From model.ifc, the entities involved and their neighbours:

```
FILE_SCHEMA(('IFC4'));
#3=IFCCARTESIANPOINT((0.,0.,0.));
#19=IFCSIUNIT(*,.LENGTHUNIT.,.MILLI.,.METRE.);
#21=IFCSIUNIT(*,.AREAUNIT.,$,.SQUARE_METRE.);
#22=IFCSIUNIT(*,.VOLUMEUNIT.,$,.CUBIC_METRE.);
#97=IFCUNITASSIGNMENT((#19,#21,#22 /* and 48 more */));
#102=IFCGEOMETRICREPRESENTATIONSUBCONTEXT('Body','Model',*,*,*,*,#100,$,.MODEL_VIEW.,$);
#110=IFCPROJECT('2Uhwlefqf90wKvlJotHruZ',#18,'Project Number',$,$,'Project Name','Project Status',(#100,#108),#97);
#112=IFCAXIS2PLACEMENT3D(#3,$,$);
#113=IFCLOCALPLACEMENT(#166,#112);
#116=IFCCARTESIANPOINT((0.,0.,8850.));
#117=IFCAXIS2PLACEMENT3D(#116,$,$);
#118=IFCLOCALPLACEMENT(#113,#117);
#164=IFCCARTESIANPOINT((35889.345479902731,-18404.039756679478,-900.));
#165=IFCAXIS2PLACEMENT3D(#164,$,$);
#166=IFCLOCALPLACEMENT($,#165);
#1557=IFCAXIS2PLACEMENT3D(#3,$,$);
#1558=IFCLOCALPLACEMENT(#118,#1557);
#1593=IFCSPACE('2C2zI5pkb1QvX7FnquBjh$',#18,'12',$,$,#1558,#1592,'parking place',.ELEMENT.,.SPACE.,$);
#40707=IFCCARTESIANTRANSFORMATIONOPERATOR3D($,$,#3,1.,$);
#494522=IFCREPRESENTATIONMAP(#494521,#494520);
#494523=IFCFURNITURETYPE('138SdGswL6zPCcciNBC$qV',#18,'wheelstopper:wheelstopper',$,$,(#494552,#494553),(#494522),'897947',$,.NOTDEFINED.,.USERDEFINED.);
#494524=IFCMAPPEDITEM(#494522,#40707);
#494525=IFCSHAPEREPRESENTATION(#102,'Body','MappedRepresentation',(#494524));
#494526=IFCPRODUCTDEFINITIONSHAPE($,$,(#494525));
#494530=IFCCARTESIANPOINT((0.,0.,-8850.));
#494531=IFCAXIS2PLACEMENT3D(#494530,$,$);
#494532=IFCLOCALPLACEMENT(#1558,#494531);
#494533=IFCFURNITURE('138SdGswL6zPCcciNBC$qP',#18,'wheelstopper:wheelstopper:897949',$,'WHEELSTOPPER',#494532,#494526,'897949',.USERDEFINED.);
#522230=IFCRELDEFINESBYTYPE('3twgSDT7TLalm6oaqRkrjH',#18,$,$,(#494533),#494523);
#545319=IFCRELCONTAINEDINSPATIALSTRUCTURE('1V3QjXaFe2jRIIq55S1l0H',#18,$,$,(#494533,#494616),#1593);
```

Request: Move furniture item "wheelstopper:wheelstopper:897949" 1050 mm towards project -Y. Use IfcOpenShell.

```python
import ifcopenshell
import ifcopenshell.api.geometry
import ifcopenshell.util.placement

model = ifcopenshell.open("model.ifc")

item = model.by_guid("138SdGswL6zPCcciNBC$qP")
matrix = ifcopenshell.util.placement.get_local_placement(item.ObjectPlacement)
matrix[1, 3] -= 1050.0
ifcopenshell.api.geometry.edit_object_placement(model, product=item, matrix=matrix, is_si=False)

print(ifcopenshell.util.placement.get_local_placement(item.ObjectPlacement).round(3) + 0.0)

model.write("model_edited.ifc")
```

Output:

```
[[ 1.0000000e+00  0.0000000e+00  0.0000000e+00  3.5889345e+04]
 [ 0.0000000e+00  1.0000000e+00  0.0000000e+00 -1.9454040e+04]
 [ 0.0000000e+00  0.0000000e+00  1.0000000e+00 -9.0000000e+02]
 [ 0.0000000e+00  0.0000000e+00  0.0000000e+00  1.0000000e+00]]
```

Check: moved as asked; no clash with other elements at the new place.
